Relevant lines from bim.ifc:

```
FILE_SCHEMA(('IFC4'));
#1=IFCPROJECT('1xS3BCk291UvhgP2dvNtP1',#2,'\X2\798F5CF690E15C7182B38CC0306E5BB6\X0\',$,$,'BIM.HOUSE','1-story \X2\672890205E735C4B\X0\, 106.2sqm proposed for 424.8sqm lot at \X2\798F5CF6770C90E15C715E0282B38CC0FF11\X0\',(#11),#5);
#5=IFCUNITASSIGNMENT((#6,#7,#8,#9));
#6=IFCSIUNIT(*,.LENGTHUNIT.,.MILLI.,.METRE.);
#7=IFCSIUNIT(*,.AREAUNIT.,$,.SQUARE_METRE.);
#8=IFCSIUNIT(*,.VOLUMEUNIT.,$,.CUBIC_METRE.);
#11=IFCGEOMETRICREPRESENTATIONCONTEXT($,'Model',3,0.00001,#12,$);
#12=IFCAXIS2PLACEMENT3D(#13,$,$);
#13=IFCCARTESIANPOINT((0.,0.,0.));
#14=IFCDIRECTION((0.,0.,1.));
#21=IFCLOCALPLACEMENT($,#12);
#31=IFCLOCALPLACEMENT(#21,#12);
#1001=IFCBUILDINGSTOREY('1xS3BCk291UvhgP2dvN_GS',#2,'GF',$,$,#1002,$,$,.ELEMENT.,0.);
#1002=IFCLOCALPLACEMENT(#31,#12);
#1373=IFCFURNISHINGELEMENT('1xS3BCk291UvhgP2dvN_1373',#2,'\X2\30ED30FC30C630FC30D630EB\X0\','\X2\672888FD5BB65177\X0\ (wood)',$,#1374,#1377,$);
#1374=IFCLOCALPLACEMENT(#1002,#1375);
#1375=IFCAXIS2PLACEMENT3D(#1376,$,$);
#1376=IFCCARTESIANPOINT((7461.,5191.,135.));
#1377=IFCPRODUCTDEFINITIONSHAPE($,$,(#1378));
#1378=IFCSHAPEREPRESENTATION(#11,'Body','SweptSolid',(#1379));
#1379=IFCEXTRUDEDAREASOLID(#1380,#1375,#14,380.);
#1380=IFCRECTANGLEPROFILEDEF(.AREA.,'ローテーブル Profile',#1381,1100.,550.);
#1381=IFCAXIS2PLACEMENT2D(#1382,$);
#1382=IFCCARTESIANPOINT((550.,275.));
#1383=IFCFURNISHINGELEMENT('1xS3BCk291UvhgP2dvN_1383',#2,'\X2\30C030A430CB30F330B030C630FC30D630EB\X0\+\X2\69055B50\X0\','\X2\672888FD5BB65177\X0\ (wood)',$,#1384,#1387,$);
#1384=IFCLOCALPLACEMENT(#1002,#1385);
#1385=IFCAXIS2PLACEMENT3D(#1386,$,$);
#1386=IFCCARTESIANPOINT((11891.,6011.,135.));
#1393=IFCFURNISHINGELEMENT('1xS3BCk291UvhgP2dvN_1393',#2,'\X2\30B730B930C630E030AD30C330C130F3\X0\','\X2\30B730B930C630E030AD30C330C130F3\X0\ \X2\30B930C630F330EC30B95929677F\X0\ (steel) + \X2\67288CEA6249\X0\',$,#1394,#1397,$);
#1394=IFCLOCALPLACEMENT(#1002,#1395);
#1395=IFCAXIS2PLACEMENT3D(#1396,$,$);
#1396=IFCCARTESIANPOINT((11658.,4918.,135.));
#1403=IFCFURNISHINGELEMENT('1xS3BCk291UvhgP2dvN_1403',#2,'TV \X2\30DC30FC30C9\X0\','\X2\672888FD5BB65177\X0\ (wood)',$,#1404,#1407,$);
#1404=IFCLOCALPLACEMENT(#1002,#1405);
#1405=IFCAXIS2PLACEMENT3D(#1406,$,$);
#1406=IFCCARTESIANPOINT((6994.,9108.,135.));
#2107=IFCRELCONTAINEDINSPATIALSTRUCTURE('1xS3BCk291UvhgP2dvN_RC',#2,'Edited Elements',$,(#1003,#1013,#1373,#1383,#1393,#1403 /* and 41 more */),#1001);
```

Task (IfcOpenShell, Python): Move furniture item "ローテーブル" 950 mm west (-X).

```python
import ifcopenshell
import ifcopenshell.api.geometry
import ifcopenshell.util.placement
import ifcopenshell.util.unit

model = ifcopenshell.open("bim.ifc")
unit_scale = ifcopenshell.util.unit.calculate_unit_scale(model)

item = model.by_guid("1xS3BCk291UvhgP2dvN_1373")
matrix = ifcopenshell.util.placement.get_local_placement(item.ObjectPlacement)
matrix[0, 3] -= 0.95 / unit_scale
ifcopenshell.api.geometry.edit_object_placement(model, product=item, matrix=matrix, is_si=False)

print(ifcopenshell.util.placement.get_local_placement(item.ObjectPlacement).round(3) + 0.0)

model.write("bim_updated.ifc")
```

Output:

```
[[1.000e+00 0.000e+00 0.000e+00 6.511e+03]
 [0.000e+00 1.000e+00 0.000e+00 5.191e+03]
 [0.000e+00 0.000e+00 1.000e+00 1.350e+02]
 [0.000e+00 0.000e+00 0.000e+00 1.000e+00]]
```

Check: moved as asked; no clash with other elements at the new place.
